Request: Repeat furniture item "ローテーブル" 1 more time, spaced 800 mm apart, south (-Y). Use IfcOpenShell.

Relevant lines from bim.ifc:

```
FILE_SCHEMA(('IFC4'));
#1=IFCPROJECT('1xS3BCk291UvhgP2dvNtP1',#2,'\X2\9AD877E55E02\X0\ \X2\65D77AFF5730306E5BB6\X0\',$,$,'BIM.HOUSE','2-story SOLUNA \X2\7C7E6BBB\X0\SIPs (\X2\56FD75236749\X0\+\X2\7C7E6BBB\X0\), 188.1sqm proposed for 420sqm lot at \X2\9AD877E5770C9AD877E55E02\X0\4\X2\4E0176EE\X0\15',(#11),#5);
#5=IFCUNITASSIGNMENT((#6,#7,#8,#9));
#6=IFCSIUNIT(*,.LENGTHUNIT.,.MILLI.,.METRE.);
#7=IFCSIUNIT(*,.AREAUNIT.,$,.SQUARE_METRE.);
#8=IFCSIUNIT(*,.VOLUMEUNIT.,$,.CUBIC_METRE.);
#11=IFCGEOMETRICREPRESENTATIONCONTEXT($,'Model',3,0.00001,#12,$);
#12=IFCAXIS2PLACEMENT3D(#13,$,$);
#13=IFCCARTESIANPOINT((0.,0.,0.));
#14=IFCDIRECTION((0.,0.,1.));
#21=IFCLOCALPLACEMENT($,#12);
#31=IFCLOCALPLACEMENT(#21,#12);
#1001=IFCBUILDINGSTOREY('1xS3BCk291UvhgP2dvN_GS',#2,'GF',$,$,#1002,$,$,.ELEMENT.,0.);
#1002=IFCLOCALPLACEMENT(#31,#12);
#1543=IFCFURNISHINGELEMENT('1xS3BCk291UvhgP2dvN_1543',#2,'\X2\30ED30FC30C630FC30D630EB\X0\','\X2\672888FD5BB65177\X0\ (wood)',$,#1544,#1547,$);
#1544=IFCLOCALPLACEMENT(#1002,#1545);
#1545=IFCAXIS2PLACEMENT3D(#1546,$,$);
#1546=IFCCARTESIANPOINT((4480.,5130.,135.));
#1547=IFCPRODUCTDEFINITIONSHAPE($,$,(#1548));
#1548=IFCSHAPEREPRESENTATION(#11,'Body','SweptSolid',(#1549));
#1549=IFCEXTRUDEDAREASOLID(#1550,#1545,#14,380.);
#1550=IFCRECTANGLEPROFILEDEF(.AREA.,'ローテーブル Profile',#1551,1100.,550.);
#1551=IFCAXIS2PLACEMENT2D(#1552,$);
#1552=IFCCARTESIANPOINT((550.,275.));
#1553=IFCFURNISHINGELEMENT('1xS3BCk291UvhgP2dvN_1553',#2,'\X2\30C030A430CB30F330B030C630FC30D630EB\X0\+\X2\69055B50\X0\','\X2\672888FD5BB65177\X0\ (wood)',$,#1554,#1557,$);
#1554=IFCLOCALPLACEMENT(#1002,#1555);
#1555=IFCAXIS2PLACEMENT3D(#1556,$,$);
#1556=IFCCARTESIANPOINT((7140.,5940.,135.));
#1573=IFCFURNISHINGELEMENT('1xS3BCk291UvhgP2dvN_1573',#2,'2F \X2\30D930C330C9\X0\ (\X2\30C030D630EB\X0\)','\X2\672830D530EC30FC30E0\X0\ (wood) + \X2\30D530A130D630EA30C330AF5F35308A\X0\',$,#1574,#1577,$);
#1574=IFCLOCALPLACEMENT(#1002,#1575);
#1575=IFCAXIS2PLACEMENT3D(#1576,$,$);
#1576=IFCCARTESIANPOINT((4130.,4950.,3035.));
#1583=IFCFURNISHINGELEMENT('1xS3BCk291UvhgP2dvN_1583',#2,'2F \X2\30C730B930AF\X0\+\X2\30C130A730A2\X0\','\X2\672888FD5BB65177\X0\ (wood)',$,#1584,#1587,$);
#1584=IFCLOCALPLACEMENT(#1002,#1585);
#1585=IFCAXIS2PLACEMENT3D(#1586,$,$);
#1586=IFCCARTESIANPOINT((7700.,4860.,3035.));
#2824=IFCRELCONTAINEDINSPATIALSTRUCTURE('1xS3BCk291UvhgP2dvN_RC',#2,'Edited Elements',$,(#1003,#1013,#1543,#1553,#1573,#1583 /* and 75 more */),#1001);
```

```python
import numpy as np
import ifcopenshell
import ifcopenshell.api.geometry
import ifcopenshell.api.root
import ifcopenshell.util.element
import ifcopenshell.util.placement
import ifcopenshell.util.unit

model = ifcopenshell.open("bim.ifc")
unit_scale = ifcopenshell.util.unit.calculate_unit_scale(model)


def reuse_history(source, copy):
    """copy_class also copies each property set's owner history, people and application; keep the originals."""
    for rel in copy.IsDefinedBy:
        if rel.is_a("IfcRelDefinesByProperties") and (history := rel.RelatingPropertyDefinition.OwnerHistory):
            rel.RelatingPropertyDefinition.OwnerHistory = source.OwnerHistory
            ifcopenshell.util.element.remove_deep2(model, history)


source = model.by_id(1543)
base = ifcopenshell.util.placement.get_local_placement(source.ObjectPlacement)
step = np.array([0.0, -1.0, 0.0]) * 0.8 / unit_scale

for i in range(1, 2):
    copy = ifcopenshell.api.root.copy_class(model, product=source)
    copy.Representation = ifcopenshell.util.element.copy_deep(
        model, source.Representation, exclude=["IfcGeometricRepresentationContext", "IfcRepresentationMap"]
    )
    reuse_history(source, copy)
    matrix = base.copy()
    matrix[:3, 3] += i * step
    print("added at", matrix[:3, 3].round(3) + 0.0)
    ifcopenshell.api.geometry.edit_object_placement(model, product=copy, matrix=matrix, is_si=False)

model.write("bim_edited.ifc")
```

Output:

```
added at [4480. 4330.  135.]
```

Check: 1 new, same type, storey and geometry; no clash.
